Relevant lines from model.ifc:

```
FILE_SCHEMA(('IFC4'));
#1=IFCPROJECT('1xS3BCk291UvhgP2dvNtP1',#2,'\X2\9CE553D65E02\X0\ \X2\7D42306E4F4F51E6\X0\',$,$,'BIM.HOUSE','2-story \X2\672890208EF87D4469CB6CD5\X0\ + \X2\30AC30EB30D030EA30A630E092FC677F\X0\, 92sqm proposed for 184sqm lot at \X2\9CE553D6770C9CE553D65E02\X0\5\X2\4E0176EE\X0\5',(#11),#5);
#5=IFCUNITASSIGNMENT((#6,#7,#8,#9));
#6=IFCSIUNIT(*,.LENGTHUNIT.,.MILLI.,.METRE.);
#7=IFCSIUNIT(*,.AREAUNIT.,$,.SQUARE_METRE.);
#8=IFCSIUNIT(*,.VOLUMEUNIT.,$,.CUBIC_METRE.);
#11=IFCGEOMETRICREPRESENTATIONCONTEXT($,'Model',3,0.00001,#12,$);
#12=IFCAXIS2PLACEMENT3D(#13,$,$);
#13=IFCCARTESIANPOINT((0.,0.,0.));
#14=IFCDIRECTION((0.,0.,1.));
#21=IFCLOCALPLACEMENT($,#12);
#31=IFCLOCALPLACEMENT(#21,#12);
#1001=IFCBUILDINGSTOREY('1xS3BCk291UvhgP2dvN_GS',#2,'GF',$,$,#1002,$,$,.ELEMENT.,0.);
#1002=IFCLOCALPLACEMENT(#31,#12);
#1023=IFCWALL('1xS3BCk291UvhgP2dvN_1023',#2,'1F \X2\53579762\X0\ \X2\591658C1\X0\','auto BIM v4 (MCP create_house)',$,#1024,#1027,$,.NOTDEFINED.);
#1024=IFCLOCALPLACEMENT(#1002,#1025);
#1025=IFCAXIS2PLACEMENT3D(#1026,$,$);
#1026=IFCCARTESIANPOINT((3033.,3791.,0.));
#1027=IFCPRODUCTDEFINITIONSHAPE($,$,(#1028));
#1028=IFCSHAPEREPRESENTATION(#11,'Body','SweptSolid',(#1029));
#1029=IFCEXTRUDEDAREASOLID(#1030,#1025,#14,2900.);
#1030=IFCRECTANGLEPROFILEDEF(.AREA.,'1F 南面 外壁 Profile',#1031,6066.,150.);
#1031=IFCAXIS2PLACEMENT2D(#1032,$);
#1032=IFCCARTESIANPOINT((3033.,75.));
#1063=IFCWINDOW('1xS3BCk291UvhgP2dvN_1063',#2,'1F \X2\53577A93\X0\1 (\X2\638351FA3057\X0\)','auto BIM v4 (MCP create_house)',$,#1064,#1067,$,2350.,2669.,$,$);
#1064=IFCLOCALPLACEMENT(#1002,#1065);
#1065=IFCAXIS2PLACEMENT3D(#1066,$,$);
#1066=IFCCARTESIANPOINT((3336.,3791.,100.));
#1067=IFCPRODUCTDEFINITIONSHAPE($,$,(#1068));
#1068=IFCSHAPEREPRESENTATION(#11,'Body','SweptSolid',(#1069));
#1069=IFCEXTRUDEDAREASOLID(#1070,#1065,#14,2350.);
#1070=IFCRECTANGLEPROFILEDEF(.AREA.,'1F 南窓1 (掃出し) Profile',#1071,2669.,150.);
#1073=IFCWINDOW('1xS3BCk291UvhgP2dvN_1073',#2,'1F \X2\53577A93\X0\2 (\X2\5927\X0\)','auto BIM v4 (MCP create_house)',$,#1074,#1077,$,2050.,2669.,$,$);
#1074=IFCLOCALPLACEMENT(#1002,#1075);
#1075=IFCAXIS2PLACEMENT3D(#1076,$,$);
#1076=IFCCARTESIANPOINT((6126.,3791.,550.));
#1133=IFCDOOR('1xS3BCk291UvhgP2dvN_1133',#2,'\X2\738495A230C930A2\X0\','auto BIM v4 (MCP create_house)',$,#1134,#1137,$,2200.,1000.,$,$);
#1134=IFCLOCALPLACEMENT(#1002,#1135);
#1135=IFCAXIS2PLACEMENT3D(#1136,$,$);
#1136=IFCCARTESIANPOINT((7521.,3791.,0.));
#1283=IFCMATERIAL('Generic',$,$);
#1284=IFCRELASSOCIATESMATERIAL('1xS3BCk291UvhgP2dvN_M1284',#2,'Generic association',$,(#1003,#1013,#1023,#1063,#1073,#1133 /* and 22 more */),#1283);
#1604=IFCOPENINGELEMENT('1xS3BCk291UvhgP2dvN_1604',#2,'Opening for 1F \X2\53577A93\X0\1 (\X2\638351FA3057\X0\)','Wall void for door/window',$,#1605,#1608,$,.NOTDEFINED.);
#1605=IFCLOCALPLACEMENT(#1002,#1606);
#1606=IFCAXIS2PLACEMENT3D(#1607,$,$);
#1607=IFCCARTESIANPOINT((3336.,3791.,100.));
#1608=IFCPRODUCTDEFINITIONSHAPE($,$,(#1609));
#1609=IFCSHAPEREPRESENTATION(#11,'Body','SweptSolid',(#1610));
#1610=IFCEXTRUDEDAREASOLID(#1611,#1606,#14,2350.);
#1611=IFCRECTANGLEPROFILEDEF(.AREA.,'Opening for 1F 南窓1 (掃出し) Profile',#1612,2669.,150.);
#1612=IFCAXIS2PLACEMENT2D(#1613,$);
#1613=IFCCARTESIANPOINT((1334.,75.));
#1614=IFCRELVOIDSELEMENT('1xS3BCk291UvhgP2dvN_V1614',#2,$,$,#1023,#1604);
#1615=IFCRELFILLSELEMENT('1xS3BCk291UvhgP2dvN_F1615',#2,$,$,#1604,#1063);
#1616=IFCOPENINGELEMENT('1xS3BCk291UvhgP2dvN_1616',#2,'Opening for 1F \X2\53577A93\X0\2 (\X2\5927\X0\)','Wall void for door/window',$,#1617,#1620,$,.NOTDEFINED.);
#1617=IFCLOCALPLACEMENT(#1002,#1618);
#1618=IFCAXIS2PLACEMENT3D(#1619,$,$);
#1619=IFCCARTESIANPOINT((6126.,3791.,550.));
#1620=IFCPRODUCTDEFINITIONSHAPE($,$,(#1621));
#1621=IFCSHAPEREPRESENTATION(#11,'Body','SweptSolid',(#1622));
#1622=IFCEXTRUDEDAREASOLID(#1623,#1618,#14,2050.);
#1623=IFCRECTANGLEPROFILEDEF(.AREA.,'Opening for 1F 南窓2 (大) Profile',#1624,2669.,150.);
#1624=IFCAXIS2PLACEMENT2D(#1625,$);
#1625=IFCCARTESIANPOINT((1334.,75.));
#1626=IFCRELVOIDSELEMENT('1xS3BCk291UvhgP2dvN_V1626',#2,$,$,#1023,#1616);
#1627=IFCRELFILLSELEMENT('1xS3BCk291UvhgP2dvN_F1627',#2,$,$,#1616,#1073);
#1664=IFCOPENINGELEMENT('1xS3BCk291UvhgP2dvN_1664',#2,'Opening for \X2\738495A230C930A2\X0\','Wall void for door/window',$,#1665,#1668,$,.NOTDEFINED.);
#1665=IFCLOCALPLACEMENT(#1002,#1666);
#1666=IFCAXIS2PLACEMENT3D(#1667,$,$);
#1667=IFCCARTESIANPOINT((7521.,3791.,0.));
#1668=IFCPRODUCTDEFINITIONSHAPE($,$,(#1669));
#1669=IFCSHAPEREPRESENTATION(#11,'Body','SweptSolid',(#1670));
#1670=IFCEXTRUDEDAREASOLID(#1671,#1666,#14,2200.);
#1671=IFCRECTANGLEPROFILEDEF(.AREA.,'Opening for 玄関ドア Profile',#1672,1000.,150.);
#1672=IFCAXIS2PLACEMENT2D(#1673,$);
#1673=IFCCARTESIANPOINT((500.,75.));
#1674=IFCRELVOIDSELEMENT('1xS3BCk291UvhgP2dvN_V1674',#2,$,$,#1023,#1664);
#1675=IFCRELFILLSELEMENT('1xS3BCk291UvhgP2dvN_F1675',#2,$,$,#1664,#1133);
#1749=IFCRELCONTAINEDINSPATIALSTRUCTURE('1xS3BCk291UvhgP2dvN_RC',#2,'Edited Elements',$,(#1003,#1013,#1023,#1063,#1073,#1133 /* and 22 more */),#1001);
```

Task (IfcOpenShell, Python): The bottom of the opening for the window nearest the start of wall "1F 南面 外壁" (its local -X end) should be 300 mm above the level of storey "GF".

```python
import numpy as np
import ifcopenshell
import ifcopenshell.api.geometry
import ifcopenshell.geom
import ifcopenshell.util.element
import ifcopenshell.util.placement
import ifcopenshell.util.shape
import ifcopenshell.util.unit

model = ifcopenshell.open("model.ifc")
unit_scale = ifcopenshell.util.unit.calculate_unit_scale(model)

window = model.by_guid("1xS3BCk291UvhgP2dvN_1063")
opening = window.FillsVoids[0].RelatingOpeningElement
storey = ifcopenshell.util.element.get_container(window, ifc_class="IfcBuildingStorey")
level = ifcopenshell.util.placement.get_local_placement(storey.ObjectPlacement)[2, 3]

# The opening's origin need not be at the sill, so measure its lowest point.
shape = ifcopenshell.geom.create_shape(ifcopenshell.geom.settings(), opening)
bottom = ifcopenshell.util.shape.get_shape_bottom_elevation(shape, shape.geometry) / unit_scale
dz = level + 0.3 / unit_scale - bottom

shift = np.array([0.0, 0.0, dz])
# The window is not placed relative to its opening, so move both.
for product in (opening, window):
    matrix = ifcopenshell.util.placement.get_local_placement(product.ObjectPlacement)
    matrix[:3, 3] += shift
    ifcopenshell.api.geometry.edit_object_placement(model, product=product, matrix=matrix, is_si=False)

print(f"moved by {dz * unit_scale:+.3f} m")

model.write("model-out.ifc")
```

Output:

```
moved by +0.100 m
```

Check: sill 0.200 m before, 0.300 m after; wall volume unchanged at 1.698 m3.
